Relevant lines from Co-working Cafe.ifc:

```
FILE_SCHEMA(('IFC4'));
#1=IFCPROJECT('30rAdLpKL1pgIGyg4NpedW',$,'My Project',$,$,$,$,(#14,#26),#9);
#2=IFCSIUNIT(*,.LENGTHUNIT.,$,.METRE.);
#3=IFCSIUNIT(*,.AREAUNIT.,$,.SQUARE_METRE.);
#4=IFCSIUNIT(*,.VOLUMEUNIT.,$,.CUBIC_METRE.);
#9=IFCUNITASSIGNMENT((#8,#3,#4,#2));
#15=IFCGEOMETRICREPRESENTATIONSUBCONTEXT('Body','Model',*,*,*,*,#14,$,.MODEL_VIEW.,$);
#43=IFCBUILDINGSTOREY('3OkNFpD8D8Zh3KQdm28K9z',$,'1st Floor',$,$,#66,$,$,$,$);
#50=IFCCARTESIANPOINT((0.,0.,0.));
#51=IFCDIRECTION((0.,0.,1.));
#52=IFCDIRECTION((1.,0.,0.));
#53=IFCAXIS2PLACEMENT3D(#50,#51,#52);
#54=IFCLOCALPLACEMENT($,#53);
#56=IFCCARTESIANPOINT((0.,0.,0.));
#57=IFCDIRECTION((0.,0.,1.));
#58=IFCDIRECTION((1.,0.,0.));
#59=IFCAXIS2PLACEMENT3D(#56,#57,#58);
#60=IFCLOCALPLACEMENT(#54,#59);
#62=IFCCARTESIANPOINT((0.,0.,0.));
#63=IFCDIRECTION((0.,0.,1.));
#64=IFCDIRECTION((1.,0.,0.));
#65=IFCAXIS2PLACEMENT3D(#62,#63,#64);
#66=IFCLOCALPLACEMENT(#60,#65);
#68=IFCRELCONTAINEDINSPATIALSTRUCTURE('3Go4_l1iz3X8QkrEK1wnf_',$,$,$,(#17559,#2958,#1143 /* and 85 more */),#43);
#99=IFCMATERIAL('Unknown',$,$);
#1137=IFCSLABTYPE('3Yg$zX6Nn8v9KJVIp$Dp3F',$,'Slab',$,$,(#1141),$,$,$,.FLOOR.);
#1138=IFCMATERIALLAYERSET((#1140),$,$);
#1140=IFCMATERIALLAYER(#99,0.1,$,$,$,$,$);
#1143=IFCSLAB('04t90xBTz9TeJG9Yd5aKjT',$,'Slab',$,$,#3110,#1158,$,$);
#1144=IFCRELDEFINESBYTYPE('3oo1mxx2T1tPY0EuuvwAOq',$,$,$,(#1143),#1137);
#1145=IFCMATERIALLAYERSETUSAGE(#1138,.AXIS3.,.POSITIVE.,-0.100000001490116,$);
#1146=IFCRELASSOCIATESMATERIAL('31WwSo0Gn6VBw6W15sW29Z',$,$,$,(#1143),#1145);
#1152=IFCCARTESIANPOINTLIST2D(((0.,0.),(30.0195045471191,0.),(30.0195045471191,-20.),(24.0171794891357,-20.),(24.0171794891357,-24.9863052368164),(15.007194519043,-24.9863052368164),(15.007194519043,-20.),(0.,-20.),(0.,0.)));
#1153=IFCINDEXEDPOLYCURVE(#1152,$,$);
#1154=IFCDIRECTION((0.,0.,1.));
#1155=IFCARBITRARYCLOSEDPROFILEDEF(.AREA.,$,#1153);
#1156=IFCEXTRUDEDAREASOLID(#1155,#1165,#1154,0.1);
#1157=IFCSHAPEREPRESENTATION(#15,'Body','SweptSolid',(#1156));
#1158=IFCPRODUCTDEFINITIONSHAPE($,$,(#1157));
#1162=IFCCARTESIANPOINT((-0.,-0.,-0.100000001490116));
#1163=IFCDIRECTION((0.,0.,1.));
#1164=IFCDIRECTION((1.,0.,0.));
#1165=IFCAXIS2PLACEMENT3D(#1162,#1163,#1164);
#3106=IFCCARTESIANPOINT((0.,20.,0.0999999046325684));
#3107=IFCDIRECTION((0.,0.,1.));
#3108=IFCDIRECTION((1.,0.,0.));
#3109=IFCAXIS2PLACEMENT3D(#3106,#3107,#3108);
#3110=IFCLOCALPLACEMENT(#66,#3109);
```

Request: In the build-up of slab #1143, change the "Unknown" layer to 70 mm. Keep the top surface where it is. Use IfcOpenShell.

```python
import ifcopenshell
import ifcopenshell.util.element
import ifcopenshell.util.representation
import ifcopenshell.util.unit

model = ifcopenshell.open("Co-working Cafe.ifc")
unit_scale = ifcopenshell.util.unit.calculate_unit_scale(model)

layer_set = model.by_id(1138)
layer = next(l for l in layer_set.MaterialLayers if l.Material and l.Material.Name == "Unknown")
change = 0.07 / unit_scale - layer.LayerThickness
layer.LayerThickness += change

# Geometry does not follow the layer set by itself.
slabs = [e for e in ifcopenshell.util.element.get_elements_by_material(model, layer_set) if e.is_a("IfcSlab")]
for slab in sorted(slabs, key=lambda e: e.id()):
    body = ifcopenshell.util.representation.get_representation(slab, "Model", "Body")
    solid = body.Items[0]
    old_depth = solid.Depth
    solid.Depth += change
    # Extruded upwards: lower the start of the extrusion so the top stays.
    x, y, z = solid.Position.Location.Coordinates
    solid.Position.Location = model.createIfcCartesianPoint((x, y, z - change))
    print(slab.id(), f"{old_depth:g} -> {solid.Depth:g}")

# The layers are counted up from the underside, which has moved.
for usage in {ifcopenshell.util.element.get_material(slab) for slab in slabs}:
    usage.OffsetFromReferenceLine -= change

model.write("Co-working Cafe_updated.ifc")
```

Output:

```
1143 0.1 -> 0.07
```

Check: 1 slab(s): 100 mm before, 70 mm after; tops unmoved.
